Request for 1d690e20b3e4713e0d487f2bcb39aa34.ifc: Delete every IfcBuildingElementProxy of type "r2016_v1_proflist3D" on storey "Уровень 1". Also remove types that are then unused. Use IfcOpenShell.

First a look at what the model holds.

```python
import ifcopenshell
import ifcopenshell.util.element

model = ifcopenshell.open("1d690e20b3e4713e0d487f2bcb39aa34.ifc")
print(model.schema)
storey = next(s for s in model.by_type("IfcBuildingStorey") if s.Name == "Уровень 1")
proxies = [e for e in ifcopenshell.util.element.get_decomposition(storey) if e.is_a("IfcBuildingElementProxy")]
seen = {}
for e in proxies:
    element_type = ifcopenshell.util.element.get_type(e)
    name = element_type.Name if element_type not in (None, e) else None
    seen[name] = seen.get(name, 0) + 1
for name, count in sorted(seen.items(), key=str):
    print(count, "x", name)
```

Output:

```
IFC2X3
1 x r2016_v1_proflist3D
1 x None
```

```python
import ifcopenshell
import ifcopenshell.api.root
import ifcopenshell.util.element

model = ifcopenshell.open("1d690e20b3e4713e0d487f2bcb39aa34.ifc")

storey = next(s for s in model.by_type("IfcBuildingStorey") if s.Name == "Уровень 1")
proxies = [e for e in ifcopenshell.util.element.get_decomposition(storey) if e.is_a("IfcBuildingElementProxy")]
targets = [e for e in proxies if (t := ifcopenshell.util.element.get_type(e)) not in (None, e) and t.Name == "r2016_v1_proflist3D"]
types = {ifcopenshell.util.element.get_type(e) for e in targets} - {None, *targets}

for e in targets:
    ifcopenshell.api.root.remove_product(model, product=e)
print(len(targets), "removed")

unused = [t for t in types if not ifcopenshell.util.element.get_types(t)]
for t in unused:
    ifcopenshell.api.root.remove_product(model, product=t)
print(len(unused), "unused types removed")

model.write("1d690e20b3e4713e0d487f2bcb39aa34-out.ifc")
```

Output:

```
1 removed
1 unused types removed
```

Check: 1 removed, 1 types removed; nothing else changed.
